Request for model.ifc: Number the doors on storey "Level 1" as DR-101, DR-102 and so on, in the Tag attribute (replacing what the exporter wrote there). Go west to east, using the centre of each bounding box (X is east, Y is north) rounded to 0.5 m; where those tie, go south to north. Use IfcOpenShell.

First a look at what the model holds.

```python
import ifcopenshell
import ifcopenshell.util.element
import ifcopenshell.util.placement

model = ifcopenshell.open("model.ifc")
print(model.schema)
storey = next(s for s in model.by_type("IfcBuildingStorey") if s.Name == "Level 1")
doors = [e for e in ifcopenshell.util.element.get_decomposition(storey) if e.is_a("IfcDoor")]
for e in sorted(doors, key=lambda e: e.id()):
    origin = ifcopenshell.util.placement.get_local_placement(e.ObjectPlacement)[:3, 3]
    print(e.id(), e.Tag, e.Name, origin.round(2) + 0.0, sep=" | ")
```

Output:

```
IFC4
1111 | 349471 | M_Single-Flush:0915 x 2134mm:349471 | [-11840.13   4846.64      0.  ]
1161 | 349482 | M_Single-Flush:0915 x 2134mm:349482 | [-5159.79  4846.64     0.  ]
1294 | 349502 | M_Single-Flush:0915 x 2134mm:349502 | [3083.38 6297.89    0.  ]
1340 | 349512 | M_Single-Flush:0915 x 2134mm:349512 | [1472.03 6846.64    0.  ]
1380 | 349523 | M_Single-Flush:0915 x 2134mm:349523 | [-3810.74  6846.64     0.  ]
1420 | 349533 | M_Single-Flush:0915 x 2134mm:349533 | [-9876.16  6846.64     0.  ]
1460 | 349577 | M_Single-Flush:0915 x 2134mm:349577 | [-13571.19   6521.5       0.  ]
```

```python
import ifcopenshell
import ifcopenshell.geom
import ifcopenshell.util.element
import ifcopenshell.util.shape

model = ifcopenshell.open("model.ifc")
settings = ifcopenshell.geom.settings()
settings.set("use-world-coords", True)


def centre(element):
    shape = ifcopenshell.geom.create_shape(settings, element)
    return ifcopenshell.util.shape.get_bbox_centroid(shape.geometry)


storey = next(s for s in model.by_type("IfcBuildingStorey") if s.Name == "Level 1")
doors = [e for e in ifcopenshell.util.element.get_decomposition(storey) if e.is_a("IfcDoor")]

# Insertion points can sit at a corner or the storey origin, so sort by the geometry (in metres).
centres = {e: centre(e) for e in doors}
doors.sort(key=lambda e: (round(centres[e][0] / 0.5), centres[e][1]))

for i, e in enumerate(doors, start=1):
    number = f"DR-1{i:02d}"
    e.Tag = number
    print(e.id(), number)

model.write("model_updated.ifc")
```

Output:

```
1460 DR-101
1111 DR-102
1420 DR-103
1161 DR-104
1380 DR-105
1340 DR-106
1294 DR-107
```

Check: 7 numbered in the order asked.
